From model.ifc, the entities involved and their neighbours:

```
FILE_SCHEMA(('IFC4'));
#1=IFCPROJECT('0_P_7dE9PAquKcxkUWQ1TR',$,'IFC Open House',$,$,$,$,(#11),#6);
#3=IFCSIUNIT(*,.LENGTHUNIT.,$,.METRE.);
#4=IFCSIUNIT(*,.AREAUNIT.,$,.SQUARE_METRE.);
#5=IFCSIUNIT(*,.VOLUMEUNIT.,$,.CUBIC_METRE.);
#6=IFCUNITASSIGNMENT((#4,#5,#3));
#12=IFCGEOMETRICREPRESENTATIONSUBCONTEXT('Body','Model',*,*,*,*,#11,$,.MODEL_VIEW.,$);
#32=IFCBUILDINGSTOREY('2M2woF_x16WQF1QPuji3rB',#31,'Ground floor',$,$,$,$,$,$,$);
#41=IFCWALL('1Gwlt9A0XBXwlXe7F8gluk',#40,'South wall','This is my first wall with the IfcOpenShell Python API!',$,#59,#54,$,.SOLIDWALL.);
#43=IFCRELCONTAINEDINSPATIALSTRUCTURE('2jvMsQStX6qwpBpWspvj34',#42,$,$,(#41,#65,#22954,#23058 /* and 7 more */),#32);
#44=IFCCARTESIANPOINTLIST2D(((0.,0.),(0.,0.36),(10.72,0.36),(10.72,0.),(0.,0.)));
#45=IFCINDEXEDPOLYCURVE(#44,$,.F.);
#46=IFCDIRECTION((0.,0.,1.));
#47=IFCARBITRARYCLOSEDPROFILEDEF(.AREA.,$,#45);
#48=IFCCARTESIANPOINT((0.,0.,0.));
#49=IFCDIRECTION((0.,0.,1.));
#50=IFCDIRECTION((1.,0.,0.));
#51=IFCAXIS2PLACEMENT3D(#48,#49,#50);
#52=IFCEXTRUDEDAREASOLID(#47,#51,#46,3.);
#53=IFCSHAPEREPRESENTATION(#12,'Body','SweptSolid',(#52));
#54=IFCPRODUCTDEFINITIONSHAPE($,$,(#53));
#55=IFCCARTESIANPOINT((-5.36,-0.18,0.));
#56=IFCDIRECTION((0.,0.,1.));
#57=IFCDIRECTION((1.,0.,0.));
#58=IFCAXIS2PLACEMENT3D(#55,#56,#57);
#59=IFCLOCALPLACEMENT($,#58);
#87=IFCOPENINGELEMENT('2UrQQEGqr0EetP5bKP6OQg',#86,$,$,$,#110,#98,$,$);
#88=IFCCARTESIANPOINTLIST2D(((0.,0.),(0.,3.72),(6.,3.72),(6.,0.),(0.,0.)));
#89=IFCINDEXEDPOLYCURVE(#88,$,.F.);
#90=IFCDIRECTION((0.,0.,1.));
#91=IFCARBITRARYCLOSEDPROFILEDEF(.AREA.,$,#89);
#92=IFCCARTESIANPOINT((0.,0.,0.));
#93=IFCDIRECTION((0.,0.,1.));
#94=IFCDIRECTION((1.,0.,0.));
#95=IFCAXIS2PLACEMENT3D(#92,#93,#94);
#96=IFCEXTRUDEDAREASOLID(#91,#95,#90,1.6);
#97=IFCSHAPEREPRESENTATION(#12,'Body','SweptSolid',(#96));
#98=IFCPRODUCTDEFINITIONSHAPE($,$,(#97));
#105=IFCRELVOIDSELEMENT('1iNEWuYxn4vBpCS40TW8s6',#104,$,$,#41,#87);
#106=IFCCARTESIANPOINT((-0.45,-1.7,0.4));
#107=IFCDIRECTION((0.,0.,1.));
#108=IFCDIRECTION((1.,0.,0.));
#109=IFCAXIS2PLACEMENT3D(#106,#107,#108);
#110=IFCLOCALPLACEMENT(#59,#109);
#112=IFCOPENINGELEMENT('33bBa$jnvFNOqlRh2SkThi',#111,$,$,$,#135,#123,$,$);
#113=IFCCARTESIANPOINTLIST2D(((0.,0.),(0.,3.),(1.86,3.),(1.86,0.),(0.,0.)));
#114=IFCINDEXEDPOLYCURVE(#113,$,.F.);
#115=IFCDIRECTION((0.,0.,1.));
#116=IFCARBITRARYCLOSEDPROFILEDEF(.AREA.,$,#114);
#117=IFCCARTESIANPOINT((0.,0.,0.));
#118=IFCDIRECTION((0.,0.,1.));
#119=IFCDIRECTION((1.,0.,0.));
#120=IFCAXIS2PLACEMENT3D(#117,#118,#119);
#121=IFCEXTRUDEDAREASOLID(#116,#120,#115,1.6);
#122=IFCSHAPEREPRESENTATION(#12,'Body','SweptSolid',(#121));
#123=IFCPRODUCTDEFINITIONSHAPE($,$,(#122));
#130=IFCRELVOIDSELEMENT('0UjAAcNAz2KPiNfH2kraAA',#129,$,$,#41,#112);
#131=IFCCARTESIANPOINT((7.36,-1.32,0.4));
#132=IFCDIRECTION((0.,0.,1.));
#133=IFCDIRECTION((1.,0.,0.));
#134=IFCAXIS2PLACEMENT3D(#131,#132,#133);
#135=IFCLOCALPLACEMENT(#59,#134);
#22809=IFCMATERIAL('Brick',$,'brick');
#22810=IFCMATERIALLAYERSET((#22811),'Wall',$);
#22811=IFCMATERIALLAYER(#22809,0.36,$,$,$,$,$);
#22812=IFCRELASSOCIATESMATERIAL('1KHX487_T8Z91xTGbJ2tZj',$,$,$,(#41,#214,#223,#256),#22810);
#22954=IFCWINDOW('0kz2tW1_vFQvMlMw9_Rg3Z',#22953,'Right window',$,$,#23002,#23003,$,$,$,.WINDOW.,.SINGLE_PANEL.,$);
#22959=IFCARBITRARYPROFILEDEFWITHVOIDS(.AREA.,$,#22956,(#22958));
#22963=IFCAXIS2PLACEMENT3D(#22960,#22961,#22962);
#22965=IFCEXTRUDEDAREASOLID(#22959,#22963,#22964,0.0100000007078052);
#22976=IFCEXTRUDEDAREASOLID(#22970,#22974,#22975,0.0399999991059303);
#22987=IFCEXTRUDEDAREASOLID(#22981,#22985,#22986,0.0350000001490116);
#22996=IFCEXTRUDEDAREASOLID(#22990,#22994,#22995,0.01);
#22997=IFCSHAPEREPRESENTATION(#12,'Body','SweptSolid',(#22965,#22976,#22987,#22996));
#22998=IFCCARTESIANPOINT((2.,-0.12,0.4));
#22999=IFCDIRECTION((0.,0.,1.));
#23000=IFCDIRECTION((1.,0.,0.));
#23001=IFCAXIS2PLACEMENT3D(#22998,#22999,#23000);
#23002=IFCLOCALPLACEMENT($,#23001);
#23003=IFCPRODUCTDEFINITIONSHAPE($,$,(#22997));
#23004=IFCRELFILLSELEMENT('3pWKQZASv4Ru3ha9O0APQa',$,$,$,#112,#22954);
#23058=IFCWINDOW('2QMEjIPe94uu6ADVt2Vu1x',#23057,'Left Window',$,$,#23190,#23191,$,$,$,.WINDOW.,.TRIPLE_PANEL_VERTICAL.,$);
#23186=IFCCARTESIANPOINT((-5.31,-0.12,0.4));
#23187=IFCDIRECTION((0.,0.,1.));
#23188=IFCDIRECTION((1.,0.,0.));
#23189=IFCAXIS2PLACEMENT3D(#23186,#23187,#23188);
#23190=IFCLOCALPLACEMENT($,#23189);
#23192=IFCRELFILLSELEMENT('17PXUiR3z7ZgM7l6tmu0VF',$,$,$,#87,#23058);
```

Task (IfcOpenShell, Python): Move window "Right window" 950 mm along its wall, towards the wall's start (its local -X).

```python
import ifcopenshell
import ifcopenshell.api.geometry
import ifcopenshell.util.placement
import ifcopenshell.util.unit

model = ifcopenshell.open("model.ifc")
unit_scale = ifcopenshell.util.unit.calculate_unit_scale(model)

window = model.by_id(22954)
opening = window.FillsVoids[0].RelatingOpeningElement
wall = opening.VoidsElements[0].RelatingBuildingElement

wall_matrix = ifcopenshell.util.placement.get_local_placement(wall.ObjectPlacement)
shift = wall_matrix[:3, 0] * -0.95 / unit_scale
before = ifcopenshell.util.placement.get_local_placement(window.ObjectPlacement)[:3, 3].copy()

# The window is not placed relative to its opening, so move both.
for product in (opening, window):
    matrix = ifcopenshell.util.placement.get_local_placement(product.ObjectPlacement)
    matrix[:3, 3] += shift
    ifcopenshell.api.geometry.edit_object_placement(model, product=product, matrix=matrix, is_si=False)

after = ifcopenshell.util.placement.get_local_placement(window.ObjectPlacement)[:3, 3]
print("window moved by", (after - before).round(3) + 0.0)

model.write("model_edited.ifc")
```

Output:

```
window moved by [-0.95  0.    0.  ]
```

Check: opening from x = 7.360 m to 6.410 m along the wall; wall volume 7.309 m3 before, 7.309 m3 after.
